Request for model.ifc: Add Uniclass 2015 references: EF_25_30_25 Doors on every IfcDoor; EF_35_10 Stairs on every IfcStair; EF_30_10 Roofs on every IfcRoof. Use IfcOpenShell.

First a look at what the model holds.

```python
import ifcopenshell

model = ifcopenshell.open("model.ifc")
print(model.schema)
print("classifications:", [c.Name for c in model.by_type("IfcClassification")])
for ifc_class in ("IfcDoor", "IfcRoof", "IfcStair", "IfcWall", "IfcWindow"):
    print(ifc_class, len(model.by_type(ifc_class)))
```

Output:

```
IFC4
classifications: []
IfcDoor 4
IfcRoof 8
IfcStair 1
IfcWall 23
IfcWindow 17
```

```python
import ifcopenshell
import ifcopenshell.api.classification

model = ifcopenshell.open("model.ifc")

system = ifcopenshell.api.classification.add_classification(model, classification="Uniclass 2015")

codes = {
    "IfcDoor": ("EF_25_30_25", "Doors"),
    "IfcStair": ("EF_35_10", "Stairs"),
    "IfcRoof": ("EF_30_10", "Roofs"),
}
for ifc_class, (code, name) in codes.items():
    products = model.by_type(ifc_class)
    ifcopenshell.api.classification.add_reference(
        model, products=products, classification=system, identification=code, name=name
    )
    print(code, len(products))

model.write("model_edited.ifc")
```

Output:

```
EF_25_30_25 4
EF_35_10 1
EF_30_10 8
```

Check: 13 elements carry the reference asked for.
